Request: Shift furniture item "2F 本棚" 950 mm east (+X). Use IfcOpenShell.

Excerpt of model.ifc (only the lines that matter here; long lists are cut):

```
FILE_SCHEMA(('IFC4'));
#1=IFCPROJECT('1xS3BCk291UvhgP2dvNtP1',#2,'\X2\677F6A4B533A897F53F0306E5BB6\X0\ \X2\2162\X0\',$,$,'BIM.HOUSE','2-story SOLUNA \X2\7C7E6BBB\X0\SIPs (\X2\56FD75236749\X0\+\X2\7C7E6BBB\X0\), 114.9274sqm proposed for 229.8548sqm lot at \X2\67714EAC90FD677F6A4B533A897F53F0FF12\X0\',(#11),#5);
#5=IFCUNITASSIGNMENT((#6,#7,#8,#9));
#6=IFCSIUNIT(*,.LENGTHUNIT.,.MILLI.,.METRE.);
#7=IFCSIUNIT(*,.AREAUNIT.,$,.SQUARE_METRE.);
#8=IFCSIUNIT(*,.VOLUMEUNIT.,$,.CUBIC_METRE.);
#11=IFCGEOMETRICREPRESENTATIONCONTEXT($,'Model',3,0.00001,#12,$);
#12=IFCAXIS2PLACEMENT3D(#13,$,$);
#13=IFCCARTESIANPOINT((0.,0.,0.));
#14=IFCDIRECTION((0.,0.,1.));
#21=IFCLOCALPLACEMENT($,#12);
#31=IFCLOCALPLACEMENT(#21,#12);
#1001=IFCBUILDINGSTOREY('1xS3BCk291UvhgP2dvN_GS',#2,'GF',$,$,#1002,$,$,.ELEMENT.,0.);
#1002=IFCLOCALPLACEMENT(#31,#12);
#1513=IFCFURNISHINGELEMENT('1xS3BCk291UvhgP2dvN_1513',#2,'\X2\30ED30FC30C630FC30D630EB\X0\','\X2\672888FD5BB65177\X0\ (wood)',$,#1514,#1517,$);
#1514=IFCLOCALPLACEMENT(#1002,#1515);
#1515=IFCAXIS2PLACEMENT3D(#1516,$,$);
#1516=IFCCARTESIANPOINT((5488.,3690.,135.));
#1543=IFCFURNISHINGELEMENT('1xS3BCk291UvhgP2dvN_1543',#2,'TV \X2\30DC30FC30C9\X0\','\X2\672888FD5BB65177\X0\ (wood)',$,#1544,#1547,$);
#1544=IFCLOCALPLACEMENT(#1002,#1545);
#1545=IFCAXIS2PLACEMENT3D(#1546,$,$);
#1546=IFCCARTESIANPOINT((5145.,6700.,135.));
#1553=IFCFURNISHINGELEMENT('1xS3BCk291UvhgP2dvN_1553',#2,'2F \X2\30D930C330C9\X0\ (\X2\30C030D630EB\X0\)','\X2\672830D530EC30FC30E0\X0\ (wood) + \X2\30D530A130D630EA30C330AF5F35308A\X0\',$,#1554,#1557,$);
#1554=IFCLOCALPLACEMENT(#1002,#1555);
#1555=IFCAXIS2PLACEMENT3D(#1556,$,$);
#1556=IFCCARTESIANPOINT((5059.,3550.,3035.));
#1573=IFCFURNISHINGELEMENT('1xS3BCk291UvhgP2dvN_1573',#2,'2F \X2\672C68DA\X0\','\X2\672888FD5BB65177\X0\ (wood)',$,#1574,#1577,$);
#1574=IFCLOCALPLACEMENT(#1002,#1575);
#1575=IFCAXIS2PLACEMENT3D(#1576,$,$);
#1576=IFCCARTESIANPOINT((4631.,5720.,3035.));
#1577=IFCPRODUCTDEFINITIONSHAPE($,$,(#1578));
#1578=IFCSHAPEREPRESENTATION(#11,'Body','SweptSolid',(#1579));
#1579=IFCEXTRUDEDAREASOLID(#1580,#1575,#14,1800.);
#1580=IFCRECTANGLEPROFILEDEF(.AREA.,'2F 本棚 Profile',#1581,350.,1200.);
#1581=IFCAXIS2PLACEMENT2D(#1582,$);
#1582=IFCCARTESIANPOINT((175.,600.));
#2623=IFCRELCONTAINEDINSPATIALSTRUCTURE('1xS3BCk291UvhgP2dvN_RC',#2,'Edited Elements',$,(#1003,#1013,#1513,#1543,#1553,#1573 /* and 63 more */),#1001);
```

```python
import ifcopenshell
import ifcopenshell.api.geometry
import ifcopenshell.util.placement
import ifcopenshell.util.unit

model = ifcopenshell.open("model.ifc")
unit_scale = ifcopenshell.util.unit.calculate_unit_scale(model)

item = model.by_guid("1xS3BCk291UvhgP2dvN_1573")
matrix = ifcopenshell.util.placement.get_local_placement(item.ObjectPlacement)
matrix[0, 3] += 0.95 / unit_scale
ifcopenshell.api.geometry.edit_object_placement(model, product=item, matrix=matrix, is_si=False)

print(ifcopenshell.util.placement.get_local_placement(item.ObjectPlacement).round(3) + 0.0)

model.write("model-out.ifc")
```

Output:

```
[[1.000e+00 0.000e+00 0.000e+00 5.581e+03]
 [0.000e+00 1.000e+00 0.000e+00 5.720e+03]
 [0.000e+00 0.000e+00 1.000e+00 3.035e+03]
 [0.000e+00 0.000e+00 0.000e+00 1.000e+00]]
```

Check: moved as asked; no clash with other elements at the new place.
